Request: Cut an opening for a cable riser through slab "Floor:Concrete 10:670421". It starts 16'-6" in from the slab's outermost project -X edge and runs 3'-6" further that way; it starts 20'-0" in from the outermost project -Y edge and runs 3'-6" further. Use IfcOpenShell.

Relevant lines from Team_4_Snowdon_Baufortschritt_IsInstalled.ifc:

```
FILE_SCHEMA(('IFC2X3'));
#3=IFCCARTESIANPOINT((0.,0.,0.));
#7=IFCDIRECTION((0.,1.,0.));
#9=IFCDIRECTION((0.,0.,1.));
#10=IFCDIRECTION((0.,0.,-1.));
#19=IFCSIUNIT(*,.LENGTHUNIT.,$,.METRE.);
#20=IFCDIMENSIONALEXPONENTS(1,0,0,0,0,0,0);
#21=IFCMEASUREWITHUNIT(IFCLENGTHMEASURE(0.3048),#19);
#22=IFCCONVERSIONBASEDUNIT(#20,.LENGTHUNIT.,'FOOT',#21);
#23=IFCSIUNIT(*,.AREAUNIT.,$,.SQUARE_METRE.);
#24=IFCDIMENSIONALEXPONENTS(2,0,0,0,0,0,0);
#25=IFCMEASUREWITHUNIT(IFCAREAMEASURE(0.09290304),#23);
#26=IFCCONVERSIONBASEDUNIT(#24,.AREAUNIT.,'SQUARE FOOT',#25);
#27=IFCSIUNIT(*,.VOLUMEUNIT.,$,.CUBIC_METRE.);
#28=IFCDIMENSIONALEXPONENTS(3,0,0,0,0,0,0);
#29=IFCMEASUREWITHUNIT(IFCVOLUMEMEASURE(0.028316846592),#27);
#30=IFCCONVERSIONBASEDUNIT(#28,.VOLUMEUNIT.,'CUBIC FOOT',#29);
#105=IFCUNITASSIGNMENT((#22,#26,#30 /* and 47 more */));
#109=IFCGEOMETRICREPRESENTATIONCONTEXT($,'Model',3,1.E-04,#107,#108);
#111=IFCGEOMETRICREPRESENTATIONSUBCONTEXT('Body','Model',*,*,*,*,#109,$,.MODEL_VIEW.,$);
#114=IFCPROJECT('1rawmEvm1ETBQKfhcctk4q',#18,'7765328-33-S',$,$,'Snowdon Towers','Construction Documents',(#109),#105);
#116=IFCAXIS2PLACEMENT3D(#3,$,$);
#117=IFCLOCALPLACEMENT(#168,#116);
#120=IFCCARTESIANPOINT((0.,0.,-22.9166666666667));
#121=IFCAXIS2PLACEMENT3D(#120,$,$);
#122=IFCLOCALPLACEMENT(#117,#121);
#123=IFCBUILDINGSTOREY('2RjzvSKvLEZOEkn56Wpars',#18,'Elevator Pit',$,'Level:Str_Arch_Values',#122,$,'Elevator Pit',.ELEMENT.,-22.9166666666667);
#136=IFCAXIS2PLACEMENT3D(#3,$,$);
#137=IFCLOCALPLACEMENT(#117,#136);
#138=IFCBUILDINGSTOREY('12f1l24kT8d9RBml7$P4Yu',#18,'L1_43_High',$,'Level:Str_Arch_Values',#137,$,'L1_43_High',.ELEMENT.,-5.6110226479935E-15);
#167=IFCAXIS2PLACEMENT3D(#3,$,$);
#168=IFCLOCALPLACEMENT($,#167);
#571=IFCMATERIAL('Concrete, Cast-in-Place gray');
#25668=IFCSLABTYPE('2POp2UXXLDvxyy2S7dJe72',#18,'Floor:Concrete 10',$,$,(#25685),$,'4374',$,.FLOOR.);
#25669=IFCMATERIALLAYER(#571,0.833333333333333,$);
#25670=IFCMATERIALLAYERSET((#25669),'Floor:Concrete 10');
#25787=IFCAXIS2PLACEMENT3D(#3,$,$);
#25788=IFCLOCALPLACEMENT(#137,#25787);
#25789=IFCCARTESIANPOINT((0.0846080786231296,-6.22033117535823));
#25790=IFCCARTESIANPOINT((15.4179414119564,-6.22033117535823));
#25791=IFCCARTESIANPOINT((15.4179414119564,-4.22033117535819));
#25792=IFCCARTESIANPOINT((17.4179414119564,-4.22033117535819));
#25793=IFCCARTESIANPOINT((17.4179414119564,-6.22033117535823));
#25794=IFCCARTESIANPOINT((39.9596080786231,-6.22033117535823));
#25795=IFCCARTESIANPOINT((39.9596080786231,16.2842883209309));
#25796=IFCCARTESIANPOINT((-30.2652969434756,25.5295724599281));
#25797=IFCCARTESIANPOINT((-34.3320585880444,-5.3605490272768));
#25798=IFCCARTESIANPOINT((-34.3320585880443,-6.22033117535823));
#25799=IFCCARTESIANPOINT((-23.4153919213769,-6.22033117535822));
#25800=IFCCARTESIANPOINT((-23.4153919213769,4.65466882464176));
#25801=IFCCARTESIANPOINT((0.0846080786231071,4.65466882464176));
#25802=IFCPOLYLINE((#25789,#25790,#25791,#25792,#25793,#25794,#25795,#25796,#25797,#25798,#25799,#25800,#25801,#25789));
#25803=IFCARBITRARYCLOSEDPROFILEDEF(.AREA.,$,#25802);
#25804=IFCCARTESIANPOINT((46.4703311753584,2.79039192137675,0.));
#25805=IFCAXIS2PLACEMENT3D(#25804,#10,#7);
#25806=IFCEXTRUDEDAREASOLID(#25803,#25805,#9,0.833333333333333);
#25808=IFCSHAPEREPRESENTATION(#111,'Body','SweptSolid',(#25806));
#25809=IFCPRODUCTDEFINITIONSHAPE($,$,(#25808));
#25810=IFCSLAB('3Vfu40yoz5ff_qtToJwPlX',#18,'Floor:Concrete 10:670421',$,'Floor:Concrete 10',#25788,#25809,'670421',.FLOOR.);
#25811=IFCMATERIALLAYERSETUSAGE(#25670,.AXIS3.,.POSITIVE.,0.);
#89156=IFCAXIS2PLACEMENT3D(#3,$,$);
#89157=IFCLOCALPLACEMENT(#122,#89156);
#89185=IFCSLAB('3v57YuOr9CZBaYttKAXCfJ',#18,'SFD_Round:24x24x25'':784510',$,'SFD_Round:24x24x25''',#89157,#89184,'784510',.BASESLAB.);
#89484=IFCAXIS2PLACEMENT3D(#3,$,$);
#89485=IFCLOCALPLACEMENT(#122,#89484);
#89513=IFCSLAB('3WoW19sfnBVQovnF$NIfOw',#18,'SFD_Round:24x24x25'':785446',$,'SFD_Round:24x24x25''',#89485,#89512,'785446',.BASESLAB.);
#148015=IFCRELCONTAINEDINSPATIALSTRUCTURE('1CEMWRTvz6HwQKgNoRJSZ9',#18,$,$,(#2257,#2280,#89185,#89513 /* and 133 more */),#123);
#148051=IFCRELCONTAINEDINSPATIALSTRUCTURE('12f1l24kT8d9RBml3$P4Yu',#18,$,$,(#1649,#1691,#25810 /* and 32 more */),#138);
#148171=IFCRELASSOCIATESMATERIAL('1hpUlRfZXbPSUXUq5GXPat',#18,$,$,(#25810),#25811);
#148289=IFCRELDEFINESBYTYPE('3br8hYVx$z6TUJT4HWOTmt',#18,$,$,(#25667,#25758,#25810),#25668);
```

```python
import numpy as np
import ifcopenshell
import ifcopenshell.api.feature
import ifcopenshell.api.geometry
import ifcopenshell.api.root
import ifcopenshell.geom
import ifcopenshell.util.placement
import ifcopenshell.util.representation
import ifcopenshell.util.shape
import ifcopenshell.util.unit

model = ifcopenshell.open("Team_4_Snowdon_Baufortschritt_IsInstalled.ifc")
unit_scale = ifcopenshell.util.unit.calculate_unit_scale(model)
settings = ifcopenshell.geom.settings()


def volume(element):
    """Net volume in cubic metres, openings subtracted."""
    shape = ifcopenshell.geom.create_shape(settings, element)
    return ifcopenshell.util.shape.get_volume(shape.geometry)


slab = model.by_guid("3Vfu40yoz5ff_qtToJwPlX")
before = volume(slab)

# Extent in the slab's own axes, in metres. The edges named are its -X and -Y sides.
slab_shape = ifcopenshell.geom.create_shape(settings, slab)
vertices = ifcopenshell.util.shape.get_vertices(slab_shape.geometry)
x_min, y_min, bottom = vertices.min(axis=0)
top = vertices[:, 2].max()

opening = ifcopenshell.api.root.create_entity(model, ifc_class="IfcOpeningElement", name="Cable riser opening")
context = ifcopenshell.util.representation.get_context(model, "Model", "Body", "MODEL_VIEW")
width, depth = 1.0668, 1.0668
outline = [(0.0, 0.0), (width, 0.0), (width, depth), (0.0, depth), (0.0, 0.0)]
# Overshoot both faces by 50 mm so the cut is clean.
shape = ifcopenshell.api.geometry.add_slab_representation(
    model, context=context, depth=top - bottom + 0.1, polyline=outline
)
ifcopenshell.api.geometry.assign_representation(model, product=opening, representation=shape)

matrix = ifcopenshell.util.placement.get_local_placement(slab.ObjectPlacement)
matrix[:, 3] = matrix @ np.append(np.array([x_min + 5.0292, y_min + 6.096, bottom - 0.05]) / unit_scale, 1.0)
ifcopenshell.api.geometry.edit_object_placement(model, product=opening, matrix=matrix, is_si=False)
ifcopenshell.api.feature.add_feature(model, feature=opening, element=slab)

after = volume(slab)

print(f"slab volume {before:.3f} -> {after:.3f} m3")

model.write("Team_4_Snowdon_Baufortschritt_IsInstalled_updated.ifc")
```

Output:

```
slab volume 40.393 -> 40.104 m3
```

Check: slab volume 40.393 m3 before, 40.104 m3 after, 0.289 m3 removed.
